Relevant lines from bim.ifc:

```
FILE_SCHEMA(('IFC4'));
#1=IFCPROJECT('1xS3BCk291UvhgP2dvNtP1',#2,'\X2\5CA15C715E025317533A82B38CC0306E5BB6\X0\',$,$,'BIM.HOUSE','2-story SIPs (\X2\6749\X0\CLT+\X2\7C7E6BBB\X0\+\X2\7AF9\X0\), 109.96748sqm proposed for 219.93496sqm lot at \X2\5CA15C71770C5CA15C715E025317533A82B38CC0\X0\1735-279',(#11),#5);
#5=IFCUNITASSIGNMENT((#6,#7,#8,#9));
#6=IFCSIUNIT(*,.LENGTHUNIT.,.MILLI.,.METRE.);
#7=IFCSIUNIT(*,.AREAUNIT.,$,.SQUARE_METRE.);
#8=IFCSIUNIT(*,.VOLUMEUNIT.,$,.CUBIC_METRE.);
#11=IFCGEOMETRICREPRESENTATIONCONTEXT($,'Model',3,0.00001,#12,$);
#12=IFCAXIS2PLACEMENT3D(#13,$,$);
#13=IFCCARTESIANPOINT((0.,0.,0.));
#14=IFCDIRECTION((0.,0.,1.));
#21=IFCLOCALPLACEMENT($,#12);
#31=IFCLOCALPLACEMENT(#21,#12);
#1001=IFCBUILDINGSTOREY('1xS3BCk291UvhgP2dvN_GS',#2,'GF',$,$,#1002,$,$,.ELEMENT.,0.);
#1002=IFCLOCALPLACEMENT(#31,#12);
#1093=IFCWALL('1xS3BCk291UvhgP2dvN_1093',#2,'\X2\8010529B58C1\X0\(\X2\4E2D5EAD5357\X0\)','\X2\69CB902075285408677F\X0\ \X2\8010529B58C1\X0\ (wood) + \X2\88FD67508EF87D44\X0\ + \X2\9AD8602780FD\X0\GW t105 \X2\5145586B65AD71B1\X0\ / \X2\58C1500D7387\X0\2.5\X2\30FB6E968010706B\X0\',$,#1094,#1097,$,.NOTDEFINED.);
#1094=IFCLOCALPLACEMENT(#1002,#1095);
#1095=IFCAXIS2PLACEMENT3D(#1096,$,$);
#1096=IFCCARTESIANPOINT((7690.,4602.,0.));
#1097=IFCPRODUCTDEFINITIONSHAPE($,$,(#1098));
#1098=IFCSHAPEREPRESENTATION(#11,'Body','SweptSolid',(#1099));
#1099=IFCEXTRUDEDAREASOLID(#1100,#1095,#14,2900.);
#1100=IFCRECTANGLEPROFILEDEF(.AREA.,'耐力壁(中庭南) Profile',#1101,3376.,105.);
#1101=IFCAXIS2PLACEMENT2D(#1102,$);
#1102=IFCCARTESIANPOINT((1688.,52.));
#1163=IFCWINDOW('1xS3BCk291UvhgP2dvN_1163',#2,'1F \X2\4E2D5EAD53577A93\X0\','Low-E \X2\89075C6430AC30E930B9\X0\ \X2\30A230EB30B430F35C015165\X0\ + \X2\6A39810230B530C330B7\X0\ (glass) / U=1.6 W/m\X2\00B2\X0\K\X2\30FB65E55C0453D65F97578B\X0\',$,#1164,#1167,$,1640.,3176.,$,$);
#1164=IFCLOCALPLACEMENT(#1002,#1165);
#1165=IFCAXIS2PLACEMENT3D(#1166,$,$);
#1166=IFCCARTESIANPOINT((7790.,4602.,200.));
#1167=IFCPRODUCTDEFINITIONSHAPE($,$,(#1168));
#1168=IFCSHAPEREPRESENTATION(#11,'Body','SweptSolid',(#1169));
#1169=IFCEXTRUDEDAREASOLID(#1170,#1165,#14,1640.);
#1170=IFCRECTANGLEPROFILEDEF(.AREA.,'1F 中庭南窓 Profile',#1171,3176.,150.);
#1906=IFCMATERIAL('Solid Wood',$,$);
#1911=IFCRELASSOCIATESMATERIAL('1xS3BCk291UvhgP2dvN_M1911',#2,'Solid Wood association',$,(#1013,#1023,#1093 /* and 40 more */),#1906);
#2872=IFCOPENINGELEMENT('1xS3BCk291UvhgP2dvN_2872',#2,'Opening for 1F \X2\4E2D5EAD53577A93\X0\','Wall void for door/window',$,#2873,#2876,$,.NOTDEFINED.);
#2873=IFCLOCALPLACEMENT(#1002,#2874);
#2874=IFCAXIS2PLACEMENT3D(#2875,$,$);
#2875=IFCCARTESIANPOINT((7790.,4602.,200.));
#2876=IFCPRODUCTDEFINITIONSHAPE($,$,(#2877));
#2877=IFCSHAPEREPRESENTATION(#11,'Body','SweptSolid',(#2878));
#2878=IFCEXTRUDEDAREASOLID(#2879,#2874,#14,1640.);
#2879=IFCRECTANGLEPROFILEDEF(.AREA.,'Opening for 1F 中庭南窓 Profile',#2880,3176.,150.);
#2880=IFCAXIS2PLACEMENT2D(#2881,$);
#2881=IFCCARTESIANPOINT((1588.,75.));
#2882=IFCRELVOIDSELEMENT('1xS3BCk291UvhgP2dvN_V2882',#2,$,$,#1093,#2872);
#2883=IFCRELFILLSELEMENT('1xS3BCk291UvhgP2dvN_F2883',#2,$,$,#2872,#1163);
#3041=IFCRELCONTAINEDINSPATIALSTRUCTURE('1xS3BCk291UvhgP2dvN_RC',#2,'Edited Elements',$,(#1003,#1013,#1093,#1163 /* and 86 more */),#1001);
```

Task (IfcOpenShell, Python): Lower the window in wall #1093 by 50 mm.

```python
import numpy as np
import ifcopenshell
import ifcopenshell.api.geometry
import ifcopenshell.util.placement
import ifcopenshell.util.unit

model = ifcopenshell.open("bim.ifc")
unit_scale = ifcopenshell.util.unit.calculate_unit_scale(model)

window = model.by_guid("1xS3BCk291UvhgP2dvN_1163")
opening = window.FillsVoids[0].RelatingOpeningElement
dz = -0.05 / unit_scale

shift = np.array([0.0, 0.0, dz])
# The window is not placed relative to its opening, so move both.
for product in (opening, window):
    matrix = ifcopenshell.util.placement.get_local_placement(product.ObjectPlacement)
    matrix[:3, 3] += shift
    ifcopenshell.api.geometry.edit_object_placement(model, product=product, matrix=matrix, is_si=False)

print(f"moved by {dz * unit_scale:+.3f} m")

model.write("bim_rev.ifc")
```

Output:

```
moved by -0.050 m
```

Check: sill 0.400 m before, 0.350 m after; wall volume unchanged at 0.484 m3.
